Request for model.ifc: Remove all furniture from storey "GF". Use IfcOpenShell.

First a look at what the model holds.

```python
import ifcopenshell
import ifcopenshell.util.element

model = ifcopenshell.open("model.ifc")
print(model.schema)
storey = next(s for s in model.by_type("IfcBuildingStorey") if s.Name == "GF")
furniture = [e for e in ifcopenshell.util.element.get_decomposition(storey) if e.is_a("IfcFurnishingElement")]
seen = {}
for e in furniture:
    element_type = ifcopenshell.util.element.get_type(e)
    name = element_type.Name if element_type not in (None, e) else None
    seen[name] = seen.get(name, 0) + 1
for name, count in sorted(seen.items(), key=str):
    print(count, "x", name)
```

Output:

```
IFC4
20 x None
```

```python
import ifcopenshell
import ifcopenshell.api.root
import ifcopenshell.util.element

model = ifcopenshell.open("model.ifc")

storey = next(s for s in model.by_type("IfcBuildingStorey") if s.Name == "GF")
furniture = [e for e in ifcopenshell.util.element.get_decomposition(storey) if e.is_a("IfcFurnishingElement")]

for e in furniture:
    ifcopenshell.api.root.remove_product(model, product=e)
print(len(furniture), "removed")

model.write("model-out.ifc")
```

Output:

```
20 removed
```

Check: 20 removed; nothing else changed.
